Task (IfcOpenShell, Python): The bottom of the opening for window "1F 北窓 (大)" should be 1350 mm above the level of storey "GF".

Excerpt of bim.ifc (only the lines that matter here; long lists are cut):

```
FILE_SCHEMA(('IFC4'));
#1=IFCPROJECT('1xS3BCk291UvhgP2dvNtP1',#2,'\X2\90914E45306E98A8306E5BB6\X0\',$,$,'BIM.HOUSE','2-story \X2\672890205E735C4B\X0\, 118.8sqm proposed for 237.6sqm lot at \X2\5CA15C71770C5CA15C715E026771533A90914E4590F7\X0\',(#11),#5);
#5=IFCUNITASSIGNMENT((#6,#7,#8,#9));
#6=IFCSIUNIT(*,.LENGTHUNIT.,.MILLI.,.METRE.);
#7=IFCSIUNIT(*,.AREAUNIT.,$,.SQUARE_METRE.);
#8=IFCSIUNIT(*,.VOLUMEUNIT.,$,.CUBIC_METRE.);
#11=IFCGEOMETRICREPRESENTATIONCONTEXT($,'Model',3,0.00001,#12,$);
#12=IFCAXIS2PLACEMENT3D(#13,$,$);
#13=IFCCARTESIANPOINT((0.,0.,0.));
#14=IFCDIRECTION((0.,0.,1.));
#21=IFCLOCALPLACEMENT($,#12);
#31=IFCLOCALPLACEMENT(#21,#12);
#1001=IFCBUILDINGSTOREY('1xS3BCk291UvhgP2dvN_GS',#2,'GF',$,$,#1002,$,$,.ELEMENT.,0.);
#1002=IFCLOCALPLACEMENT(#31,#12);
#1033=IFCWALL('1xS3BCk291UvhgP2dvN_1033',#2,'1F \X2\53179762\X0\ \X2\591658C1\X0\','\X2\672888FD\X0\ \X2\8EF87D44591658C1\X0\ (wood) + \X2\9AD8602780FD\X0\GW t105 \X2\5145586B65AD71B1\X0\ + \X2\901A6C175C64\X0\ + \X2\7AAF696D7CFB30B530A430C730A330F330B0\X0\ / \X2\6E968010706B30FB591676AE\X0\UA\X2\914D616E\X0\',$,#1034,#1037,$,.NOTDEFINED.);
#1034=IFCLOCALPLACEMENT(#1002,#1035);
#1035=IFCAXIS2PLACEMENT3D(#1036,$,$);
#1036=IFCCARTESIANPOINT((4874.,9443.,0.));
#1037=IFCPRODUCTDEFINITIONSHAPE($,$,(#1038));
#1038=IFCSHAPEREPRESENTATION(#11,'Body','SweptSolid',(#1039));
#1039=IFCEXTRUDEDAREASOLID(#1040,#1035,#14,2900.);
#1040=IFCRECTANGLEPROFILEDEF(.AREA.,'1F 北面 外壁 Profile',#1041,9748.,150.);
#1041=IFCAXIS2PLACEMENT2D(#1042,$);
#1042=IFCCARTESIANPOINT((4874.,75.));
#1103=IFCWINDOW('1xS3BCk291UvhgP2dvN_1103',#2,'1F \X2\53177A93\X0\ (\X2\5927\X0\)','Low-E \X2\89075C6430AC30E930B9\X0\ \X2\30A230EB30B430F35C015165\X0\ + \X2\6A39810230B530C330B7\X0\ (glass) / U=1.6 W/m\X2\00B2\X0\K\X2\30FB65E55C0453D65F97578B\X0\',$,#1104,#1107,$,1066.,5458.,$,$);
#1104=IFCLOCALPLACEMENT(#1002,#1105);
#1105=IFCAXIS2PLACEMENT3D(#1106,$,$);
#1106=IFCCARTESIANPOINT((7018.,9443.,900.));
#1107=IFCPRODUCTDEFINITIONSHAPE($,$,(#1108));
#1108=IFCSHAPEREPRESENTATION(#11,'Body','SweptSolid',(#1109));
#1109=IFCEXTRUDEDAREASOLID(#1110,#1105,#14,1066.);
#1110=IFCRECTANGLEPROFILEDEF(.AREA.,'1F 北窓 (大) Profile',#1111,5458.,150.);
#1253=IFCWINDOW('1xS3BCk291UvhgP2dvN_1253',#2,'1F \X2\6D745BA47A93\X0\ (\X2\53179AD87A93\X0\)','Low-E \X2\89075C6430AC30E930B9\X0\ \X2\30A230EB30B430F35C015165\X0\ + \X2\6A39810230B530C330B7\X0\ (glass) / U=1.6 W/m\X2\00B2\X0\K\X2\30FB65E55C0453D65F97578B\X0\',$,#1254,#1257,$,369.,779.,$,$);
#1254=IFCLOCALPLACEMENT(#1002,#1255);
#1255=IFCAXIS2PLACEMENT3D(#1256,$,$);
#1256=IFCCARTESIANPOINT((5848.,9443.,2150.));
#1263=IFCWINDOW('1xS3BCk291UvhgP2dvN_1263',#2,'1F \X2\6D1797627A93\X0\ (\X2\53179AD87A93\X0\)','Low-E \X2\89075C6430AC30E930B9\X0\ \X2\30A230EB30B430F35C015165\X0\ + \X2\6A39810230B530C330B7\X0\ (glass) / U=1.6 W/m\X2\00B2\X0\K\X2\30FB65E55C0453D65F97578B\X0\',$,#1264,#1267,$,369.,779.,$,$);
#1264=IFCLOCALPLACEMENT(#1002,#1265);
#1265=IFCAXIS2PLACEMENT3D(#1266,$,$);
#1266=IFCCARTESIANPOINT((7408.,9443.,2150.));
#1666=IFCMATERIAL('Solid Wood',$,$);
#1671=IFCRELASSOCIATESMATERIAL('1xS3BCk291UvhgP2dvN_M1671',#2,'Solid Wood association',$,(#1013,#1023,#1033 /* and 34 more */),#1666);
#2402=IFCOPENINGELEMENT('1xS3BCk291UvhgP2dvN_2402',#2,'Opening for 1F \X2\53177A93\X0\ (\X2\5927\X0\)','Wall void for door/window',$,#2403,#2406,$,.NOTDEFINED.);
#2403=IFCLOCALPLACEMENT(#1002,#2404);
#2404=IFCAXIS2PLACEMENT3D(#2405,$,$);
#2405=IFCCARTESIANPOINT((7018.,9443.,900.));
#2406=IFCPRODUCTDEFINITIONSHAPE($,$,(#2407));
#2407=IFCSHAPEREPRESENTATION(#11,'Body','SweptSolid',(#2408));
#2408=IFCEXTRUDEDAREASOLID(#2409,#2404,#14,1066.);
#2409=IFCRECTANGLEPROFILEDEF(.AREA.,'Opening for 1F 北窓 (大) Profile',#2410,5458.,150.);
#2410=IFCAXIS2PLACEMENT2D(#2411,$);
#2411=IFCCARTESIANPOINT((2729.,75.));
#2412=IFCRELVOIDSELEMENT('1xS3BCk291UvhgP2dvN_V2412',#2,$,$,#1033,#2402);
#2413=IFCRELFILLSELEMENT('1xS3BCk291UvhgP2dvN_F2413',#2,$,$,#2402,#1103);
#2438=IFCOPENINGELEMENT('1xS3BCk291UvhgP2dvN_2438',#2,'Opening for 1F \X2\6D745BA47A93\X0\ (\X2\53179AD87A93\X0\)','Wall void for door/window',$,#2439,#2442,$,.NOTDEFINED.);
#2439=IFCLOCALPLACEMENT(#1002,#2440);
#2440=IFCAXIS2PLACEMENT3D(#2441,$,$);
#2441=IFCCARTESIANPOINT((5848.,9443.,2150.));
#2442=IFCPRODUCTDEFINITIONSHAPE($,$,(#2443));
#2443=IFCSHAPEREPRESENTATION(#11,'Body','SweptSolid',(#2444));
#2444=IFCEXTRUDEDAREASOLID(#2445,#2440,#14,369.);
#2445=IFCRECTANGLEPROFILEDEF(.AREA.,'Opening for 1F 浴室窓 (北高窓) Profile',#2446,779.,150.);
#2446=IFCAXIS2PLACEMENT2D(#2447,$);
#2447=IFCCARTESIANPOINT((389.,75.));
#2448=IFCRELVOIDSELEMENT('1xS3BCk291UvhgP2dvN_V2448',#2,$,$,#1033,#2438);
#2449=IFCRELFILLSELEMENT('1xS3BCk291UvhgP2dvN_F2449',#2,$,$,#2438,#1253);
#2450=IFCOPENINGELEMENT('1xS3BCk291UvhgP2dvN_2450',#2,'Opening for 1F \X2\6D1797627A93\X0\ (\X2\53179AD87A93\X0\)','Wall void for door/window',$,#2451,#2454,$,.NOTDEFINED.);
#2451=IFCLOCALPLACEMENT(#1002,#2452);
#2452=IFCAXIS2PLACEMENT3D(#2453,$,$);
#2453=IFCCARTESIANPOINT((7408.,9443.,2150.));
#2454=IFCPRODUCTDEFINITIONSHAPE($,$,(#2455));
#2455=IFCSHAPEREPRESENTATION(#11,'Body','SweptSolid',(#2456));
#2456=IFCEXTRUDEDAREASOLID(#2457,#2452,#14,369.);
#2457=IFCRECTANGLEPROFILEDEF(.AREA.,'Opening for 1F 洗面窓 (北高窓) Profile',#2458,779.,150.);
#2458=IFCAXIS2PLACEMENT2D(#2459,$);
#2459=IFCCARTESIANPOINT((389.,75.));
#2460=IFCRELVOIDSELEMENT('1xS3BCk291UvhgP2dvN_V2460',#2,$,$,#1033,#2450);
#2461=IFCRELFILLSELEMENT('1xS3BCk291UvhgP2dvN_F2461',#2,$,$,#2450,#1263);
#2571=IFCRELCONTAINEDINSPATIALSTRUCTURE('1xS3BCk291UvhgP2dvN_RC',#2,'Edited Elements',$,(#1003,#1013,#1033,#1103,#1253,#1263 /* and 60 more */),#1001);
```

```python
import numpy as np
import ifcopenshell
import ifcopenshell.api.geometry
import ifcopenshell.geom
import ifcopenshell.util.element
import ifcopenshell.util.placement
import ifcopenshell.util.shape
import ifcopenshell.util.unit

model = ifcopenshell.open("bim.ifc")
unit_scale = ifcopenshell.util.unit.calculate_unit_scale(model)

window = model.by_guid("1xS3BCk291UvhgP2dvN_1103")
opening = window.FillsVoids[0].RelatingOpeningElement
storey = ifcopenshell.util.element.get_container(window, ifc_class="IfcBuildingStorey")
level = ifcopenshell.util.placement.get_local_placement(storey.ObjectPlacement)[2, 3]

# The opening's origin need not be at the sill, so measure its lowest point.
shape = ifcopenshell.geom.create_shape(ifcopenshell.geom.settings(), opening)
bottom = ifcopenshell.util.shape.get_shape_bottom_elevation(shape, shape.geometry) / unit_scale
dz = level + 1350.0 - bottom

shift = np.array([0.0, 0.0, dz])
# The window is not placed relative to its opening, so move both.
for product in (opening, window):
    matrix = ifcopenshell.util.placement.get_local_placement(product.ObjectPlacement)
    matrix[:3, 3] += shift
    ifcopenshell.api.geometry.edit_object_placement(model, product=product, matrix=matrix, is_si=False)

print(f"moved by {dz * unit_scale:+.3f} m")

model.write("bim_rev.ifc")
```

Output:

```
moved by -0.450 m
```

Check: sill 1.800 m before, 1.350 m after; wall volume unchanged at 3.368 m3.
